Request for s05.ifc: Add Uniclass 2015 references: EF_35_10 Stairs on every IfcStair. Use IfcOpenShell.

First a look at what the model holds.

```python
import ifcopenshell

model = ifcopenshell.open("s05.ifc")
print(model.schema)
print("classifications:", [c.Name for c in model.by_type("IfcClassification")])
for ifc_class in ("IfcDoor", "IfcRoof", "IfcStair", "IfcWall", "IfcWindow"):
    print(ifc_class, len(model.by_type(ifc_class)))
```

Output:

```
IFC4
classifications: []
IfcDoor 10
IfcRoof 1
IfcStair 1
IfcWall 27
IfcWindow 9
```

```python
import ifcopenshell
import ifcopenshell.api.classification

model = ifcopenshell.open("s05.ifc")

system = ifcopenshell.api.classification.add_classification(model, classification="Uniclass 2015")

codes = {
    "IfcStair": ("EF_35_10", "Stairs"),
}
for ifc_class, (code, name) in codes.items():
    products = model.by_type(ifc_class)
    ifcopenshell.api.classification.add_reference(
        model, products=products, classification=system, identification=code, name=name
    )
    print(code, len(products))

model.write("s05-out.ifc")
```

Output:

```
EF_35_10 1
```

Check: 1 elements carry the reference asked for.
